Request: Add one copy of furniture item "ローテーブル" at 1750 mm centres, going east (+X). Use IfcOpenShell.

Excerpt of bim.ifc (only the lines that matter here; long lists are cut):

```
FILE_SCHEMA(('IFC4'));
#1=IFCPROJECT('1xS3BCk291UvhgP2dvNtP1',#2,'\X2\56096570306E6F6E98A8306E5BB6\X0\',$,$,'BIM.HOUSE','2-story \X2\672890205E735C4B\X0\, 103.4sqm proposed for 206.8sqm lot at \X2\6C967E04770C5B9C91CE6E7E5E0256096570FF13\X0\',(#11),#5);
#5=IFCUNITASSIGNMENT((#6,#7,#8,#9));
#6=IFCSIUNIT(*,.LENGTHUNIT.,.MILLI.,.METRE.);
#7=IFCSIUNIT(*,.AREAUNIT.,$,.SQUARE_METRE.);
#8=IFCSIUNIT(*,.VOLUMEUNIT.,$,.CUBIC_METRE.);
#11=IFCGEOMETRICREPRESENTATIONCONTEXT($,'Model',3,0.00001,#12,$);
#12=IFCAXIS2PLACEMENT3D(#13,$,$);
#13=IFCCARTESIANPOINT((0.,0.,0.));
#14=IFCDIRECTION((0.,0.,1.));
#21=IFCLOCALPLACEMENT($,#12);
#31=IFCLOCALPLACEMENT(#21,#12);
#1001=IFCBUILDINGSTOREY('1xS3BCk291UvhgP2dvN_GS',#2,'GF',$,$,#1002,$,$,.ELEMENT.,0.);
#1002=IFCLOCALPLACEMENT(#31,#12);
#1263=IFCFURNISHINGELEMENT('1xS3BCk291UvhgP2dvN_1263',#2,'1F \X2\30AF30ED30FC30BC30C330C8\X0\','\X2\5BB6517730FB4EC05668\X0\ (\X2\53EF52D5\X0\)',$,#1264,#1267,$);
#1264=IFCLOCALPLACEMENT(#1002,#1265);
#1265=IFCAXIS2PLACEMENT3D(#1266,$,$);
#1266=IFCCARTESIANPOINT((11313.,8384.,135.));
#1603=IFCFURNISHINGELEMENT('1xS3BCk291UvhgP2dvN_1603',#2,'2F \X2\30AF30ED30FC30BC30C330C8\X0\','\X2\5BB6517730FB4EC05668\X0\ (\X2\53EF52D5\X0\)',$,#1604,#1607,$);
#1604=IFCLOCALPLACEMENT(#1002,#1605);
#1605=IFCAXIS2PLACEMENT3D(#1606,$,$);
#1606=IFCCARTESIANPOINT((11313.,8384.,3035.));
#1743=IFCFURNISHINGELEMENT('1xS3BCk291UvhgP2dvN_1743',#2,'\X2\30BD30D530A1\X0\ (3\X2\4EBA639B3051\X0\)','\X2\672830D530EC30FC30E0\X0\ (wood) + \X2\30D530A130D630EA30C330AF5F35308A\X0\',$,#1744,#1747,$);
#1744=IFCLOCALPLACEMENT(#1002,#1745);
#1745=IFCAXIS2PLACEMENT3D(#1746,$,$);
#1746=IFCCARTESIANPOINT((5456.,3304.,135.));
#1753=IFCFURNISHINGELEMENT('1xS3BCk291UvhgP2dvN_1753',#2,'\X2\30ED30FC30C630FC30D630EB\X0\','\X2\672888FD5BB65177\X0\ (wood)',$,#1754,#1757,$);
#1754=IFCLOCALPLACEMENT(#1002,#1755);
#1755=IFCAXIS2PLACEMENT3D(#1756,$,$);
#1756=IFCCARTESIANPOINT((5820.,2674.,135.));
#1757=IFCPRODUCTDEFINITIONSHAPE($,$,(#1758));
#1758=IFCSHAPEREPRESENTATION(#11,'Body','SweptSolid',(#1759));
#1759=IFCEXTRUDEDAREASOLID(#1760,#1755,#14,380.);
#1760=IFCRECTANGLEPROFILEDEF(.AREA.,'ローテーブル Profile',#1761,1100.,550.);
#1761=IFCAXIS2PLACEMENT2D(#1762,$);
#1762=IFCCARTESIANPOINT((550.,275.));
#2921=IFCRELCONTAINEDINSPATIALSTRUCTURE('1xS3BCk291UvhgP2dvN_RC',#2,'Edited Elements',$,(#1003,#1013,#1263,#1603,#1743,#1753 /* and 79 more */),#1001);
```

```python
import numpy as np
import ifcopenshell
import ifcopenshell.api.geometry
import ifcopenshell.api.root
import ifcopenshell.util.element
import ifcopenshell.util.placement
import ifcopenshell.util.unit

model = ifcopenshell.open("bim.ifc")
unit_scale = ifcopenshell.util.unit.calculate_unit_scale(model)


def reuse_history(source, copy):
    """copy_class also copies each property set's owner history, people and application; keep the originals."""
    for rel in copy.IsDefinedBy:
        if rel.is_a("IfcRelDefinesByProperties") and (history := rel.RelatingPropertyDefinition.OwnerHistory):
            rel.RelatingPropertyDefinition.OwnerHistory = source.OwnerHistory
            ifcopenshell.util.element.remove_deep2(model, history)


source = model.by_guid("1xS3BCk291UvhgP2dvN_1753")
base = ifcopenshell.util.placement.get_local_placement(source.ObjectPlacement)
step = np.array([1.0, 0.0, 0.0]) * 1.75 / unit_scale

for i in range(1, 2):
    copy = ifcopenshell.api.root.copy_class(model, product=source)
    copy.Representation = ifcopenshell.util.element.copy_deep(
        model, source.Representation, exclude=["IfcGeometricRepresentationContext", "IfcRepresentationMap"]
    )
    reuse_history(source, copy)
    matrix = base.copy()
    matrix[:3, 3] += i * step
    print("added at", matrix[:3, 3].round(3) + 0.0)
    ifcopenshell.api.geometry.edit_object_placement(model, product=copy, matrix=matrix, is_si=False)

model.write("bim-out.ifc")
```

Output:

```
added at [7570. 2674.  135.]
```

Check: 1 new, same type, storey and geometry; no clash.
